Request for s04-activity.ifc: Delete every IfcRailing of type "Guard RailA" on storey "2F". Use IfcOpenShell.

First a look at what the model holds.

```python
import ifcopenshell
import ifcopenshell.util.element

model = ifcopenshell.open("s04-activity.ifc")
print(model.schema)
storey = next(s for s in model.by_type("IfcBuildingStorey") if s.Name == "2F")
railings = [e for e in ifcopenshell.util.element.get_decomposition(storey) if e.is_a("IfcRailing")]
seen = {}
for e in railings:
    element_type = ifcopenshell.util.element.get_type(e)
    name = element_type.Name if element_type not in (None, e) else None
    seen[name] = seen.get(name, 0) + 1
for name, count in sorted(seen.items(), key=str):
    print(count, "x", name)
```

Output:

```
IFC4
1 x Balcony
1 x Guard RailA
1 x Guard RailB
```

```python
import ifcopenshell
import ifcopenshell.api.root
import ifcopenshell.util.element

model = ifcopenshell.open("s04-activity.ifc")

storey = next(s for s in model.by_type("IfcBuildingStorey") if s.Name == "2F")
railings = [e for e in ifcopenshell.util.element.get_decomposition(storey) if e.is_a("IfcRailing")]
targets = [e for e in railings if (t := ifcopenshell.util.element.get_type(e)) not in (None, e) and t.Name == "Guard RailA"]

for e in targets:
    ifcopenshell.api.root.remove_product(model, product=e)
print(len(targets), "removed")

model.write("s04-activity_edited.ifc")
```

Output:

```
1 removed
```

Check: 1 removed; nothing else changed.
